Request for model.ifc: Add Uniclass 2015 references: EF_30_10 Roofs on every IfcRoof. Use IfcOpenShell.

First a look at what the model holds.

```python
import ifcopenshell

model = ifcopenshell.open("model.ifc")
print(model.schema)
print("classifications:", [c.Name for c in model.by_type("IfcClassification")])
for ifc_class in ("IfcDoor", "IfcRoof", "IfcStair", "IfcWall", "IfcWindow"):
    print(ifc_class, len(model.by_type(ifc_class)))
```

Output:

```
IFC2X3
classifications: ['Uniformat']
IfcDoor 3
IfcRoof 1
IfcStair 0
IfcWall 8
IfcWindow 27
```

```python
import ifcopenshell
import ifcopenshell.api.classification

model = ifcopenshell.open("model.ifc")

# IFC2X3 requires Source and Edition and has no link from the project to the system.
system = model.create_entity("IfcClassification", Source="NBS", Edition="2015", Name="Uniclass 2015")

codes = {
    "IfcRoof": ("EF_30_10", "Roofs"),
}
for ifc_class, (code, name) in codes.items():
    products = model.by_type(ifc_class)
    ifcopenshell.api.classification.add_reference(
        model, products=products, classification=system, identification=code, name=name
    )
    print(code, len(products))

model.write("model_rev.ifc")
```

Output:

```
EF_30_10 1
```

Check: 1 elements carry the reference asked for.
